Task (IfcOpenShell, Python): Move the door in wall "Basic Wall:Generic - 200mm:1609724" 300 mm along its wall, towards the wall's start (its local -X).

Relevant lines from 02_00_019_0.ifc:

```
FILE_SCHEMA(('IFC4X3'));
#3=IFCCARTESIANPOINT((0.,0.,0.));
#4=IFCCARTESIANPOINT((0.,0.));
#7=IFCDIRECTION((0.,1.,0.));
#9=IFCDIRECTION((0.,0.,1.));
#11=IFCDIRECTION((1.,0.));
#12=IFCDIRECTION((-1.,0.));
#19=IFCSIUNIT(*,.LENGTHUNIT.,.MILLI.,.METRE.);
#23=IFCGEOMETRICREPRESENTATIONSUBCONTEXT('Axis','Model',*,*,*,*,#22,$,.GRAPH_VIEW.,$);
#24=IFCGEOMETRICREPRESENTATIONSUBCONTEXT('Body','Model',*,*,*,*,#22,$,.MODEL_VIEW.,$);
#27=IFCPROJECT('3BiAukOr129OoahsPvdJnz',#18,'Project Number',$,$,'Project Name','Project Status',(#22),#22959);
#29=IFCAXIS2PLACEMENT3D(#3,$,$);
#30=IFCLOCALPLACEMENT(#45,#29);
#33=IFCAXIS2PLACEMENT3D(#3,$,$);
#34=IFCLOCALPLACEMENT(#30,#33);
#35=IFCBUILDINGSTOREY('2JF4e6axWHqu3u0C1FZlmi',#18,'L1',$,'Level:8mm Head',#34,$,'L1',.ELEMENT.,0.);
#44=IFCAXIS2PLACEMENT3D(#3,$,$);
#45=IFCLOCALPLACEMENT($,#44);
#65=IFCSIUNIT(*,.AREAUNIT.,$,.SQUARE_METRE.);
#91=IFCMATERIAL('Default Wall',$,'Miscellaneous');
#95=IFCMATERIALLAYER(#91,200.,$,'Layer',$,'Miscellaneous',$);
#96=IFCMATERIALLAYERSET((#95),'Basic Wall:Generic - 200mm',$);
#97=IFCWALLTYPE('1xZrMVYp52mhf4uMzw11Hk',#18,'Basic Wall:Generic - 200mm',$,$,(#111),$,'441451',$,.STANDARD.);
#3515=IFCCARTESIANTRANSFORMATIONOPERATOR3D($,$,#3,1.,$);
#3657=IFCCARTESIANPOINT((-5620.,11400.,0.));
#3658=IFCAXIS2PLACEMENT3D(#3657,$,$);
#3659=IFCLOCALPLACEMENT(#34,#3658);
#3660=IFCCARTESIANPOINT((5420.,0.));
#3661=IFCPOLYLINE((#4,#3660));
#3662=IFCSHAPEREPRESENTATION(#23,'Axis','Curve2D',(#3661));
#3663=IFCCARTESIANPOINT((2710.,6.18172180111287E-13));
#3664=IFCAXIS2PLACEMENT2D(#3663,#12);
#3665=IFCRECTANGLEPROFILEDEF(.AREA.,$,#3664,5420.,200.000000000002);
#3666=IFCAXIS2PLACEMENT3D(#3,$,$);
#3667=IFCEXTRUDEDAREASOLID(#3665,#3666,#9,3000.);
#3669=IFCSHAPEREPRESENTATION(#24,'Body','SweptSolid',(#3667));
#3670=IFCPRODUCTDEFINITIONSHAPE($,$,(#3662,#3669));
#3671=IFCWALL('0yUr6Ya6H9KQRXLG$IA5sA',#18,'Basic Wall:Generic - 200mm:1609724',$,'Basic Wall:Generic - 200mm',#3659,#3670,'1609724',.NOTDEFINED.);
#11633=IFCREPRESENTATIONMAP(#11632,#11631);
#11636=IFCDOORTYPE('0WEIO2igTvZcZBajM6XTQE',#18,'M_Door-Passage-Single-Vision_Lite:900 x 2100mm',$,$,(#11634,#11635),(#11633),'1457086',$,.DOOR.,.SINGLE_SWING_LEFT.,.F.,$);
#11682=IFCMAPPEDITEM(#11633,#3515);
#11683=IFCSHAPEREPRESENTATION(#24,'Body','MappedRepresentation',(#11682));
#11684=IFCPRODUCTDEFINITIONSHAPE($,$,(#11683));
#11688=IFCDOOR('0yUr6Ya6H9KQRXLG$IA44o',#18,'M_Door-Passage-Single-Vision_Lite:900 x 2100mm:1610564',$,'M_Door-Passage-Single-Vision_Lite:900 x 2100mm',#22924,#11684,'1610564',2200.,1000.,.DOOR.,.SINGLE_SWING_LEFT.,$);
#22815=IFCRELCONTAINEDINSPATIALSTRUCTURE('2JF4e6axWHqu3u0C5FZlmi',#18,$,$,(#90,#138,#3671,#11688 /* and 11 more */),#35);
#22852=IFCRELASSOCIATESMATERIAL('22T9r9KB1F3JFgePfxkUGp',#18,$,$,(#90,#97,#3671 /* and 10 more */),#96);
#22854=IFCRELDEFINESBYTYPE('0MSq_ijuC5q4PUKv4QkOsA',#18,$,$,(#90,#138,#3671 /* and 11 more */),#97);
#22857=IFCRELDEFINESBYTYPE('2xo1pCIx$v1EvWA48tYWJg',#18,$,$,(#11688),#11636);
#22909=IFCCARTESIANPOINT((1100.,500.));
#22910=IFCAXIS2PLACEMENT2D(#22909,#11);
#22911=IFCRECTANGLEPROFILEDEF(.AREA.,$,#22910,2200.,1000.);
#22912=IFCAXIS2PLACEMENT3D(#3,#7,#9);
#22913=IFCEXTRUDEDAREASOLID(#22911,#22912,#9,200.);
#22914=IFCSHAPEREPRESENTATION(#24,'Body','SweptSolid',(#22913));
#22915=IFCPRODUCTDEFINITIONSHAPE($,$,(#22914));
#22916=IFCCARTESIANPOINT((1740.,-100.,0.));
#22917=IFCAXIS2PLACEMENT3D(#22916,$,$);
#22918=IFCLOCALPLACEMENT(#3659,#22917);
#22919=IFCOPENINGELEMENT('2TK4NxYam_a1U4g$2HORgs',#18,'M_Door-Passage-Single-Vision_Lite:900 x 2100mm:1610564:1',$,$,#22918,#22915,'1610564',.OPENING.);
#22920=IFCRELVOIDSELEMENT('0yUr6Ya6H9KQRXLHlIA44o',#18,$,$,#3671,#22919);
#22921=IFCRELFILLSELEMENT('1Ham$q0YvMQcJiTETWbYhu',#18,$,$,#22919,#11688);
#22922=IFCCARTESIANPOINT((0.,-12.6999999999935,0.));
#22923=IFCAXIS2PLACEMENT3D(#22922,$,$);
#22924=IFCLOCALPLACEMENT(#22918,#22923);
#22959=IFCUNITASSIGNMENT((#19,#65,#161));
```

```python
import ifcopenshell
import ifcopenshell.api.geometry
import ifcopenshell.util.placement
import ifcopenshell.util.unit

model = ifcopenshell.open("02_00_019_0.ifc")
unit_scale = ifcopenshell.util.unit.calculate_unit_scale(model)

door = model.by_guid("0yUr6Ya6H9KQRXLG$IA44o")
opening = door.FillsVoids[0].RelatingOpeningElement
wall = opening.VoidsElements[0].RelatingBuildingElement

wall_matrix = ifcopenshell.util.placement.get_local_placement(wall.ObjectPlacement)
shift = wall_matrix[:3, 0] * -0.3 / unit_scale
before = ifcopenshell.util.placement.get_local_placement(door.ObjectPlacement)[:3, 3].copy()

# The door is placed relative to its opening, so it follows when the opening moves.
matrix = ifcopenshell.util.placement.get_local_placement(opening.ObjectPlacement)
matrix[:3, 3] += shift
ifcopenshell.api.geometry.edit_object_placement(
    model, product=opening, matrix=matrix, is_si=False, should_transform_children=True
)

after = ifcopenshell.util.placement.get_local_placement(door.ObjectPlacement)[:3, 3]
print("door moved by", (after - before).round(3) + 0.0)

model.write("02_00_019_0_v2.ifc")
```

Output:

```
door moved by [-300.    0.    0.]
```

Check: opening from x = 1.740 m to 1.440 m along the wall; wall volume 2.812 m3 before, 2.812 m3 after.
